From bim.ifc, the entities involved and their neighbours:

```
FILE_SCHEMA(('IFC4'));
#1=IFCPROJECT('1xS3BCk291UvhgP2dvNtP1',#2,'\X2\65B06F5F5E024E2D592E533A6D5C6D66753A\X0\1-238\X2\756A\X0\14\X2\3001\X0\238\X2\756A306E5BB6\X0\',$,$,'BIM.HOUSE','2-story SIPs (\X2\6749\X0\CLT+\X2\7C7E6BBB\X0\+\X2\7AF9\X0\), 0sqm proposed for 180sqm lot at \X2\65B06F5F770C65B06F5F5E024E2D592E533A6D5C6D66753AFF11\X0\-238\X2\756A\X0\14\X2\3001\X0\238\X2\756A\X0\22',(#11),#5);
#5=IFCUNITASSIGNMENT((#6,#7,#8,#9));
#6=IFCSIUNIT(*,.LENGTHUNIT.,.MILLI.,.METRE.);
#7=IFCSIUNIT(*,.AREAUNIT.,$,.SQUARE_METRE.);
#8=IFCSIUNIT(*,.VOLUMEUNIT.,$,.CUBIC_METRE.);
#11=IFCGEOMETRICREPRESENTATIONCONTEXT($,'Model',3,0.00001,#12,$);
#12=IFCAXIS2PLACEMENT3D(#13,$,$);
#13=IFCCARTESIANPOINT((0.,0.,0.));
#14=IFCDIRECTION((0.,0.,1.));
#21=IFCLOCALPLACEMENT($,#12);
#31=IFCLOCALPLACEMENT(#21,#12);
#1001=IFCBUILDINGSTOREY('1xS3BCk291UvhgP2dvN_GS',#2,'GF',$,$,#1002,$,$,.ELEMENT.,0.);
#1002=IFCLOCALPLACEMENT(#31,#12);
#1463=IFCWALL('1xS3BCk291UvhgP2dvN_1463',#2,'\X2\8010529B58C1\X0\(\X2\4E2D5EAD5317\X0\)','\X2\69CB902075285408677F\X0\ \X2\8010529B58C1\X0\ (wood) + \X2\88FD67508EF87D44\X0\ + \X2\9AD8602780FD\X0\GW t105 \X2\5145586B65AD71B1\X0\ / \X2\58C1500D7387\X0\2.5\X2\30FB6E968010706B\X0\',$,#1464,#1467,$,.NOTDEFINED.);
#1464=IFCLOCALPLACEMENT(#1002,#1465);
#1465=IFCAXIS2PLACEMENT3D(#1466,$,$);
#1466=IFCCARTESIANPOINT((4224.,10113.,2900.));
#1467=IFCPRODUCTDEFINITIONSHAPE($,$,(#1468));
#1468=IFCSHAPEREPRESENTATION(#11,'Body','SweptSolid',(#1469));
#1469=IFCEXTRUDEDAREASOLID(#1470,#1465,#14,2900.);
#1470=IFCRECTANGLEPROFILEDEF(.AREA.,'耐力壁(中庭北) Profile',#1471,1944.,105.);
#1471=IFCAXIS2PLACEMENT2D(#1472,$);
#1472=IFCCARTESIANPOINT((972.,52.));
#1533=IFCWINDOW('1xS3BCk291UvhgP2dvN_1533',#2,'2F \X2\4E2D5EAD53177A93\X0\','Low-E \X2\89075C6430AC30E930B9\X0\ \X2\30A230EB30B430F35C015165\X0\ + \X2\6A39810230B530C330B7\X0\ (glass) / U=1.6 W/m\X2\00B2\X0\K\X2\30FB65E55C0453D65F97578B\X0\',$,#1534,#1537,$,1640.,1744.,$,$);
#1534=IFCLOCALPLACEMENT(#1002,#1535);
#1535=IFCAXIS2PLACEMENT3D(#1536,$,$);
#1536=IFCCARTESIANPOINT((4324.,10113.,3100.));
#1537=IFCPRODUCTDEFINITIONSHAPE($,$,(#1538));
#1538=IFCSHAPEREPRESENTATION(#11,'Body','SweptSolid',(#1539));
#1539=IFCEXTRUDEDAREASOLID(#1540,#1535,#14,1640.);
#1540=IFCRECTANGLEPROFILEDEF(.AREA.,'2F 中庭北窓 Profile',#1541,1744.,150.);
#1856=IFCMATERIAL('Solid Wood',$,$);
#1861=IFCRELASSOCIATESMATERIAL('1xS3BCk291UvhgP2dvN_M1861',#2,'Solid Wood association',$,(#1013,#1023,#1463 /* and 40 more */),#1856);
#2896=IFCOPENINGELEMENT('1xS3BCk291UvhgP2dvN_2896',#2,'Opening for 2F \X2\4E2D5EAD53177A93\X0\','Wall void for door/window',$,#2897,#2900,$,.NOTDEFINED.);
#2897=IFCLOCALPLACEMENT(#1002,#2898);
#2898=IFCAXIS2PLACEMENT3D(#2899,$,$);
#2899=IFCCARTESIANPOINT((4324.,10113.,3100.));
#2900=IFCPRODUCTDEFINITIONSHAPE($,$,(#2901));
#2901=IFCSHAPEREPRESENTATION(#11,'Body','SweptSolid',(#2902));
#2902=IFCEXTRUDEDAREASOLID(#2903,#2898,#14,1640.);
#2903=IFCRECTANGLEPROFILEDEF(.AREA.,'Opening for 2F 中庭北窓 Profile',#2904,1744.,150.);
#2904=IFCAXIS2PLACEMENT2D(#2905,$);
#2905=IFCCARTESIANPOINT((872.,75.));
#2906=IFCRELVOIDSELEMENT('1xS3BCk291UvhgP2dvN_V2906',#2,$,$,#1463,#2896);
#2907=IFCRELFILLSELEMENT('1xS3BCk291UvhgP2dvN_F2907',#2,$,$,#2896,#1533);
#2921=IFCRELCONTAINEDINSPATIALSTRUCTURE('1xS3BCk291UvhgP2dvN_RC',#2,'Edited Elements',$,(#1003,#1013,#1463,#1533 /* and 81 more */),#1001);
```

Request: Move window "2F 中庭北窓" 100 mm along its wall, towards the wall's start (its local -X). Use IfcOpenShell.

```python
import ifcopenshell
import ifcopenshell.api.geometry
import ifcopenshell.util.placement
import ifcopenshell.util.unit

model = ifcopenshell.open("bim.ifc")
unit_scale = ifcopenshell.util.unit.calculate_unit_scale(model)

window = model.by_guid("1xS3BCk291UvhgP2dvN_1533")
opening = window.FillsVoids[0].RelatingOpeningElement
wall = opening.VoidsElements[0].RelatingBuildingElement

wall_matrix = ifcopenshell.util.placement.get_local_placement(wall.ObjectPlacement)
shift = wall_matrix[:3, 0] * -0.1 / unit_scale
before = ifcopenshell.util.placement.get_local_placement(window.ObjectPlacement)[:3, 3].copy()

# The window is not placed relative to its opening, so move both.
for product in (opening, window):
    matrix = ifcopenshell.util.placement.get_local_placement(product.ObjectPlacement)
    matrix[:3, 3] += shift
    ifcopenshell.api.geometry.edit_object_placement(model, product=product, matrix=matrix, is_si=False)

after = ifcopenshell.util.placement.get_local_placement(window.ObjectPlacement)[:3, 3]
print("window moved by", (after - before).round(3) + 0.0)

model.write("bim_v2.ifc")
```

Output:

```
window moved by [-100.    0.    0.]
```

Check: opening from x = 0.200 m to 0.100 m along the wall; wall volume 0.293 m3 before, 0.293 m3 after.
